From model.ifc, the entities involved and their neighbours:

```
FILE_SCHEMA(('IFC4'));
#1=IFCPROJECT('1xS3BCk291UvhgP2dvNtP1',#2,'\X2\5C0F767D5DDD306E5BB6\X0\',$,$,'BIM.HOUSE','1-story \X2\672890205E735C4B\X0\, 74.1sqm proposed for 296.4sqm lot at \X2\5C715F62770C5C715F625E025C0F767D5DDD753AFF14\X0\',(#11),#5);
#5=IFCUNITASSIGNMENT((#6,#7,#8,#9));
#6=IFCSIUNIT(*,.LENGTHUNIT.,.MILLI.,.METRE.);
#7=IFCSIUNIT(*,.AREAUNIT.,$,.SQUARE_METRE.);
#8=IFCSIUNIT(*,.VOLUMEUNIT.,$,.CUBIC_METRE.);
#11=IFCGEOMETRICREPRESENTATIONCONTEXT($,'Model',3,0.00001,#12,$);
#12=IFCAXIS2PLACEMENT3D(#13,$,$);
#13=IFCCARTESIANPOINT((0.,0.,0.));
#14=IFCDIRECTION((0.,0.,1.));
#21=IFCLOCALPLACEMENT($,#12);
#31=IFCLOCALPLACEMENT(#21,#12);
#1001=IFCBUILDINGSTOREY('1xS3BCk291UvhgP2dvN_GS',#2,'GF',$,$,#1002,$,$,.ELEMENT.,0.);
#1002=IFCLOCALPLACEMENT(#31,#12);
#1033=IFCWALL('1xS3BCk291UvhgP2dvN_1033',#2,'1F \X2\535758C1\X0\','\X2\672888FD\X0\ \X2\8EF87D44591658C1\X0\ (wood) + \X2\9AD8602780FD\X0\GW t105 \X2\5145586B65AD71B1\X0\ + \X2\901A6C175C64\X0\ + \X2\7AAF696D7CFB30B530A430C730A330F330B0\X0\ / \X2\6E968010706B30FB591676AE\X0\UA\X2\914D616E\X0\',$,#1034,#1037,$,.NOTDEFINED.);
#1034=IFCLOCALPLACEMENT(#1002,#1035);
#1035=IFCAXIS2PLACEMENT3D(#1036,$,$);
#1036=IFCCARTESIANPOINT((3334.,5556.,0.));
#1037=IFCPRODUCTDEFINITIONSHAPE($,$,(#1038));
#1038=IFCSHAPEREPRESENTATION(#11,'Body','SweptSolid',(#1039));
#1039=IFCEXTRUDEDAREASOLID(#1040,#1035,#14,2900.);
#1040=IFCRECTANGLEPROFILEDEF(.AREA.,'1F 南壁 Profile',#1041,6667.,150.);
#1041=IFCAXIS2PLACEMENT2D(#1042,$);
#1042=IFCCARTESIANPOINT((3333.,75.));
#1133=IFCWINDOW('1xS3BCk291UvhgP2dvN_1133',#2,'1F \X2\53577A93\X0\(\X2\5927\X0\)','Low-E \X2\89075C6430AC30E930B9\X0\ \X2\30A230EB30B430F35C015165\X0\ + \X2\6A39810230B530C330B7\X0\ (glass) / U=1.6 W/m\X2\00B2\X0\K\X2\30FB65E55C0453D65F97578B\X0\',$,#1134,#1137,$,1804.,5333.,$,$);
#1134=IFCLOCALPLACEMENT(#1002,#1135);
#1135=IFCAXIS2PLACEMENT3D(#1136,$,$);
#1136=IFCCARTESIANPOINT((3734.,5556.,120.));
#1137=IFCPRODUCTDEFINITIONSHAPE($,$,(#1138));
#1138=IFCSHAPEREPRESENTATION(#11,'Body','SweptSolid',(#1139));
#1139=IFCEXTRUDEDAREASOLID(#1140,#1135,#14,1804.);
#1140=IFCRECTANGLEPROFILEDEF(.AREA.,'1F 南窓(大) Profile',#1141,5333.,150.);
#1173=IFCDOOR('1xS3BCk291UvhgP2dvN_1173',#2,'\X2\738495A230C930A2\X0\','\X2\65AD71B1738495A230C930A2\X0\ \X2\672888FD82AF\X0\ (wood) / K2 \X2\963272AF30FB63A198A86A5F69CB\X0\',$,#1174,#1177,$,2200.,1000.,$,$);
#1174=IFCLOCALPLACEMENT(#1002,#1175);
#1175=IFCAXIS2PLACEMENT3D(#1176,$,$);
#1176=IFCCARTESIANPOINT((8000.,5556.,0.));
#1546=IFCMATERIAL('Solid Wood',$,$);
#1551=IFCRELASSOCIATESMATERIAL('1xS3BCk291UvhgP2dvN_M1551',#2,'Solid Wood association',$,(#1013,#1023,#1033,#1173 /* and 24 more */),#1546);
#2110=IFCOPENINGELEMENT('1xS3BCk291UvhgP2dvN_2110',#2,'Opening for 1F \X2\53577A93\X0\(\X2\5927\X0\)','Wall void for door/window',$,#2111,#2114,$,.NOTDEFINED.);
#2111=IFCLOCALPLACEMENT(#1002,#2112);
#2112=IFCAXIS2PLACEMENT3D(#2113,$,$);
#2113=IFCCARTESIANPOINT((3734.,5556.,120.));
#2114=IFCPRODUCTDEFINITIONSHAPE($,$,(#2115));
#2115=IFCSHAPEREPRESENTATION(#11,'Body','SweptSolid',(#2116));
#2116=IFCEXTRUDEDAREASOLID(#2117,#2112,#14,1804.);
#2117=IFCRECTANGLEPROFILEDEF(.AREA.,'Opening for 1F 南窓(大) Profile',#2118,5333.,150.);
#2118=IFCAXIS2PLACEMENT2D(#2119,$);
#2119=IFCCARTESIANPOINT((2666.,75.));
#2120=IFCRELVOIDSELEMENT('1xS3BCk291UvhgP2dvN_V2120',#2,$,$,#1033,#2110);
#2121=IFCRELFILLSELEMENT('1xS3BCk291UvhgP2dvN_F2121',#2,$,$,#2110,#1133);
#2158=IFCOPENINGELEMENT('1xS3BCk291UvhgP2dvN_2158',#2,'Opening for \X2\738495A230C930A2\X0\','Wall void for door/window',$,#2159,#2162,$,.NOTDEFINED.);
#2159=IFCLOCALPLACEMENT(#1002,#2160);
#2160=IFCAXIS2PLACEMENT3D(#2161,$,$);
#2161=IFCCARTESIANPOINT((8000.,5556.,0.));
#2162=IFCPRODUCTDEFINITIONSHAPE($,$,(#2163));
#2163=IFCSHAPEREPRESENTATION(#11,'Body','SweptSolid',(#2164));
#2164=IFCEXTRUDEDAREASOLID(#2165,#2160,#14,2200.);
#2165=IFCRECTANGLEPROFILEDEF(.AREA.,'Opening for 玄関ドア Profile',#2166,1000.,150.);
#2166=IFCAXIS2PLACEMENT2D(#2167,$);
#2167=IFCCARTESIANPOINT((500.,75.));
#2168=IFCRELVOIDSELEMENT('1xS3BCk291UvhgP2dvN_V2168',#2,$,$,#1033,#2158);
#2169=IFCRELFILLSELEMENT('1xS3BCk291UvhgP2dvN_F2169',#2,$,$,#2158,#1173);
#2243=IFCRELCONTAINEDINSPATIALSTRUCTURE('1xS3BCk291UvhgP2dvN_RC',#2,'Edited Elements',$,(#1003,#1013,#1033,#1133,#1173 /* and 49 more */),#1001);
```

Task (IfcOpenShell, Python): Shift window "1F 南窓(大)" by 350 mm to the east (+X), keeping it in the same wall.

```python
import ifcopenshell
import ifcopenshell.api.geometry
import ifcopenshell.util.placement
import ifcopenshell.util.unit

model = ifcopenshell.open("model.ifc")
unit_scale = ifcopenshell.util.unit.calculate_unit_scale(model)

window = model.by_guid("1xS3BCk291UvhgP2dvN_1133")
opening = window.FillsVoids[0].RelatingOpeningElement
wall = opening.VoidsElements[0].RelatingBuildingElement

wall_matrix = ifcopenshell.util.placement.get_local_placement(wall.ObjectPlacement)
shift = wall_matrix[:3, 0] * 0.35 / unit_scale
before = ifcopenshell.util.placement.get_local_placement(window.ObjectPlacement)[:3, 3].copy()

# The window is not placed relative to its opening, so move both.
for product in (opening, window):
    matrix = ifcopenshell.util.placement.get_local_placement(product.ObjectPlacement)
    matrix[:3, 3] += shift
    ifcopenshell.api.geometry.edit_object_placement(model, product=product, matrix=matrix, is_si=False)

after = ifcopenshell.util.placement.get_local_placement(window.ObjectPlacement)[:3, 3]
print("window moved by", (after - before).round(3) + 0.0)

model.write("model_updated.ifc")
```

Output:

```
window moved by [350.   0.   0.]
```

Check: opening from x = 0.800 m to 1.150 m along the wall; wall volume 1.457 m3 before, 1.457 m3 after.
